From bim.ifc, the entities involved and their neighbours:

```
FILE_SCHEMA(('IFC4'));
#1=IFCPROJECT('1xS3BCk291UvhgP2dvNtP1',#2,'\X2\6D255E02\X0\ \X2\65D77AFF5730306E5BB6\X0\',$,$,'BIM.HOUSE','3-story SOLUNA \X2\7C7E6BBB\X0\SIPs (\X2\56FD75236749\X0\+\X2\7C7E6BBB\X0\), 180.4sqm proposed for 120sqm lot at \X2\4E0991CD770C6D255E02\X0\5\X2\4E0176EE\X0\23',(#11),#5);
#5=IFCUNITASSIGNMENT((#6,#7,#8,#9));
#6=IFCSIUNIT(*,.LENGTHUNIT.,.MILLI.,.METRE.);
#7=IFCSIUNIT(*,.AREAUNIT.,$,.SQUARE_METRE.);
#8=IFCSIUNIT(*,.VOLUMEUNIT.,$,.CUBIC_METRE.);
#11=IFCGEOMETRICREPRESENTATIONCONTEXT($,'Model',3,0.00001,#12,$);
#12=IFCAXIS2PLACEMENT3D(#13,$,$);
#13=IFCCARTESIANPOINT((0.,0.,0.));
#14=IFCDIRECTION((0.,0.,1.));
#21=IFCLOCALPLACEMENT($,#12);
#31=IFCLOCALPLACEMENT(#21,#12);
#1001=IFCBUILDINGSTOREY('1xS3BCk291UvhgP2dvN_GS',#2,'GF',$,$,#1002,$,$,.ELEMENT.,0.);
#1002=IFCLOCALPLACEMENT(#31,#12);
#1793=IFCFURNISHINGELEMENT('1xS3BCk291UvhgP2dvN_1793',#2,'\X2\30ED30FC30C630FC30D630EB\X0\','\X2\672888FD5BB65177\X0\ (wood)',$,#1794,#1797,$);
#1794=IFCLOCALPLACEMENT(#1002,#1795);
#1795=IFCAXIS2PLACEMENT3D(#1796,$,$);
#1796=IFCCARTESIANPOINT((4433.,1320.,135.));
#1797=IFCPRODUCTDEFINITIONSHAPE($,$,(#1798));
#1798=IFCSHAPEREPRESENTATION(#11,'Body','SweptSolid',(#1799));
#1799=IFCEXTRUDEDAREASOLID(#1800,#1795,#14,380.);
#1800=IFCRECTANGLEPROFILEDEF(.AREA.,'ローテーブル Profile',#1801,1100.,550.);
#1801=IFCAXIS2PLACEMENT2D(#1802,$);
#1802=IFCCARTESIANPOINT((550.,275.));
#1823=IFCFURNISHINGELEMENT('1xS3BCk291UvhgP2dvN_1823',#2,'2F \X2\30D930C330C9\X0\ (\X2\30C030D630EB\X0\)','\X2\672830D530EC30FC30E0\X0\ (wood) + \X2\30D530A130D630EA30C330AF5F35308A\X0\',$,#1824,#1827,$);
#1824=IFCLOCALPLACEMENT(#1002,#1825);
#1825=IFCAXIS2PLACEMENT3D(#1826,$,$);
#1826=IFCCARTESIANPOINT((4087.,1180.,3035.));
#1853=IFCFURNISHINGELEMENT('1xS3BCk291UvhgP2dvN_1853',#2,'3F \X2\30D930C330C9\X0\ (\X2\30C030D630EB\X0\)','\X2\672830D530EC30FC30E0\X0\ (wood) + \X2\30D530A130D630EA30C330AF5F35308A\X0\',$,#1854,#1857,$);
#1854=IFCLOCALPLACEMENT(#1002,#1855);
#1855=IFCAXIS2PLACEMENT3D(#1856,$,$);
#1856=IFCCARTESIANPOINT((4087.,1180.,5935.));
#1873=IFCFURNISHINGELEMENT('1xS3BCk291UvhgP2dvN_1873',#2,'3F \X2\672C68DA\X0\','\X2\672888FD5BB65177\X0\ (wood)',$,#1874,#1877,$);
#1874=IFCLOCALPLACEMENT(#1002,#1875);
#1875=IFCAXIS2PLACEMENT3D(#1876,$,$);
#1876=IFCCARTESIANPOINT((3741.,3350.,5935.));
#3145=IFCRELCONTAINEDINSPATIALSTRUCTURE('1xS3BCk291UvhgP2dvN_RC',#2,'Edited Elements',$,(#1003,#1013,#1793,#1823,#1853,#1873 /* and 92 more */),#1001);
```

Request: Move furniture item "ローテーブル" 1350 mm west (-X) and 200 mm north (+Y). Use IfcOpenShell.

```python
import ifcopenshell
import ifcopenshell.api.geometry
import ifcopenshell.util.placement
import ifcopenshell.util.unit

model = ifcopenshell.open("bim.ifc")
unit_scale = ifcopenshell.util.unit.calculate_unit_scale(model)

item = model.by_guid("1xS3BCk291UvhgP2dvN_1793")
matrix = ifcopenshell.util.placement.get_local_placement(item.ObjectPlacement)
matrix[0, 3] -= 1.35 / unit_scale
matrix[1, 3] += 0.2 / unit_scale
ifcopenshell.api.geometry.edit_object_placement(model, product=item, matrix=matrix, is_si=False)

print(ifcopenshell.util.placement.get_local_placement(item.ObjectPlacement).round(3) + 0.0)

model.write("bim_updated.ifc")
```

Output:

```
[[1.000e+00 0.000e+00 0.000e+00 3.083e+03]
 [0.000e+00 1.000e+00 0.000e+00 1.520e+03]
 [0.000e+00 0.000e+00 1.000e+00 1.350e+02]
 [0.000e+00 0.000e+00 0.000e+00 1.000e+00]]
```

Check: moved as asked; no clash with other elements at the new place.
